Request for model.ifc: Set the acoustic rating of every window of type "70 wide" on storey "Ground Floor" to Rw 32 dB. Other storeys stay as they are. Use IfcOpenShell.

First a look at what the model holds.

```python
import ifcopenshell
import ifcopenshell.util.element

model = ifcopenshell.open("model.ifc")
print(model.schema)
storey = next(s for s in model.by_type("IfcBuildingStorey") if s.Name == "Ground Floor")
windows = [e for e in ifcopenshell.util.element.get_decomposition(storey) if e.is_a("IfcWindow")]
seen = {}
for e in windows:
    element_type = ifcopenshell.util.element.get_type(e)
    key = (element_type.Name if element_type != e and element_type else None, ifcopenshell.util.element.get_pset(e, "Pset_WindowCommon", "AcousticRating"))
    seen[key] = seen.get(key, 0) + 1
for (name, value), count in sorted(seen.items(), key=str):
    print(count, "x", name, "|", value)
```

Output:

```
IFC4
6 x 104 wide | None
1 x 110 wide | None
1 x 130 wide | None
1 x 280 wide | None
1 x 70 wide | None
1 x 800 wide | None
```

```python
import ifcopenshell
import ifcopenshell.api.pset
import ifcopenshell.util.element

model = ifcopenshell.open("model.ifc")

storey = next(s for s in model.by_type("IfcBuildingStorey") if s.Name == "Ground Floor")
windows = [e for e in ifcopenshell.util.element.get_decomposition(storey) if e.is_a("IfcWindow")]

count = 0
for e in windows:
    element_type = ifcopenshell.util.element.get_type(e)
    if element_type in (None, e) or element_type.Name != "70 wide":
        continue
    # add_pset returns the element's existing set when there is one.
    pset = ifcopenshell.api.pset.add_pset(model, product=e, name="Pset_WindowCommon")
    ifcopenshell.api.pset.edit_pset(model, pset=pset, properties={"AcousticRating": "Rw 32 dB"})
    count += 1

print(count, "windows updated")

model.write("model-out.ifc")
```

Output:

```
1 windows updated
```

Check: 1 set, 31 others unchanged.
